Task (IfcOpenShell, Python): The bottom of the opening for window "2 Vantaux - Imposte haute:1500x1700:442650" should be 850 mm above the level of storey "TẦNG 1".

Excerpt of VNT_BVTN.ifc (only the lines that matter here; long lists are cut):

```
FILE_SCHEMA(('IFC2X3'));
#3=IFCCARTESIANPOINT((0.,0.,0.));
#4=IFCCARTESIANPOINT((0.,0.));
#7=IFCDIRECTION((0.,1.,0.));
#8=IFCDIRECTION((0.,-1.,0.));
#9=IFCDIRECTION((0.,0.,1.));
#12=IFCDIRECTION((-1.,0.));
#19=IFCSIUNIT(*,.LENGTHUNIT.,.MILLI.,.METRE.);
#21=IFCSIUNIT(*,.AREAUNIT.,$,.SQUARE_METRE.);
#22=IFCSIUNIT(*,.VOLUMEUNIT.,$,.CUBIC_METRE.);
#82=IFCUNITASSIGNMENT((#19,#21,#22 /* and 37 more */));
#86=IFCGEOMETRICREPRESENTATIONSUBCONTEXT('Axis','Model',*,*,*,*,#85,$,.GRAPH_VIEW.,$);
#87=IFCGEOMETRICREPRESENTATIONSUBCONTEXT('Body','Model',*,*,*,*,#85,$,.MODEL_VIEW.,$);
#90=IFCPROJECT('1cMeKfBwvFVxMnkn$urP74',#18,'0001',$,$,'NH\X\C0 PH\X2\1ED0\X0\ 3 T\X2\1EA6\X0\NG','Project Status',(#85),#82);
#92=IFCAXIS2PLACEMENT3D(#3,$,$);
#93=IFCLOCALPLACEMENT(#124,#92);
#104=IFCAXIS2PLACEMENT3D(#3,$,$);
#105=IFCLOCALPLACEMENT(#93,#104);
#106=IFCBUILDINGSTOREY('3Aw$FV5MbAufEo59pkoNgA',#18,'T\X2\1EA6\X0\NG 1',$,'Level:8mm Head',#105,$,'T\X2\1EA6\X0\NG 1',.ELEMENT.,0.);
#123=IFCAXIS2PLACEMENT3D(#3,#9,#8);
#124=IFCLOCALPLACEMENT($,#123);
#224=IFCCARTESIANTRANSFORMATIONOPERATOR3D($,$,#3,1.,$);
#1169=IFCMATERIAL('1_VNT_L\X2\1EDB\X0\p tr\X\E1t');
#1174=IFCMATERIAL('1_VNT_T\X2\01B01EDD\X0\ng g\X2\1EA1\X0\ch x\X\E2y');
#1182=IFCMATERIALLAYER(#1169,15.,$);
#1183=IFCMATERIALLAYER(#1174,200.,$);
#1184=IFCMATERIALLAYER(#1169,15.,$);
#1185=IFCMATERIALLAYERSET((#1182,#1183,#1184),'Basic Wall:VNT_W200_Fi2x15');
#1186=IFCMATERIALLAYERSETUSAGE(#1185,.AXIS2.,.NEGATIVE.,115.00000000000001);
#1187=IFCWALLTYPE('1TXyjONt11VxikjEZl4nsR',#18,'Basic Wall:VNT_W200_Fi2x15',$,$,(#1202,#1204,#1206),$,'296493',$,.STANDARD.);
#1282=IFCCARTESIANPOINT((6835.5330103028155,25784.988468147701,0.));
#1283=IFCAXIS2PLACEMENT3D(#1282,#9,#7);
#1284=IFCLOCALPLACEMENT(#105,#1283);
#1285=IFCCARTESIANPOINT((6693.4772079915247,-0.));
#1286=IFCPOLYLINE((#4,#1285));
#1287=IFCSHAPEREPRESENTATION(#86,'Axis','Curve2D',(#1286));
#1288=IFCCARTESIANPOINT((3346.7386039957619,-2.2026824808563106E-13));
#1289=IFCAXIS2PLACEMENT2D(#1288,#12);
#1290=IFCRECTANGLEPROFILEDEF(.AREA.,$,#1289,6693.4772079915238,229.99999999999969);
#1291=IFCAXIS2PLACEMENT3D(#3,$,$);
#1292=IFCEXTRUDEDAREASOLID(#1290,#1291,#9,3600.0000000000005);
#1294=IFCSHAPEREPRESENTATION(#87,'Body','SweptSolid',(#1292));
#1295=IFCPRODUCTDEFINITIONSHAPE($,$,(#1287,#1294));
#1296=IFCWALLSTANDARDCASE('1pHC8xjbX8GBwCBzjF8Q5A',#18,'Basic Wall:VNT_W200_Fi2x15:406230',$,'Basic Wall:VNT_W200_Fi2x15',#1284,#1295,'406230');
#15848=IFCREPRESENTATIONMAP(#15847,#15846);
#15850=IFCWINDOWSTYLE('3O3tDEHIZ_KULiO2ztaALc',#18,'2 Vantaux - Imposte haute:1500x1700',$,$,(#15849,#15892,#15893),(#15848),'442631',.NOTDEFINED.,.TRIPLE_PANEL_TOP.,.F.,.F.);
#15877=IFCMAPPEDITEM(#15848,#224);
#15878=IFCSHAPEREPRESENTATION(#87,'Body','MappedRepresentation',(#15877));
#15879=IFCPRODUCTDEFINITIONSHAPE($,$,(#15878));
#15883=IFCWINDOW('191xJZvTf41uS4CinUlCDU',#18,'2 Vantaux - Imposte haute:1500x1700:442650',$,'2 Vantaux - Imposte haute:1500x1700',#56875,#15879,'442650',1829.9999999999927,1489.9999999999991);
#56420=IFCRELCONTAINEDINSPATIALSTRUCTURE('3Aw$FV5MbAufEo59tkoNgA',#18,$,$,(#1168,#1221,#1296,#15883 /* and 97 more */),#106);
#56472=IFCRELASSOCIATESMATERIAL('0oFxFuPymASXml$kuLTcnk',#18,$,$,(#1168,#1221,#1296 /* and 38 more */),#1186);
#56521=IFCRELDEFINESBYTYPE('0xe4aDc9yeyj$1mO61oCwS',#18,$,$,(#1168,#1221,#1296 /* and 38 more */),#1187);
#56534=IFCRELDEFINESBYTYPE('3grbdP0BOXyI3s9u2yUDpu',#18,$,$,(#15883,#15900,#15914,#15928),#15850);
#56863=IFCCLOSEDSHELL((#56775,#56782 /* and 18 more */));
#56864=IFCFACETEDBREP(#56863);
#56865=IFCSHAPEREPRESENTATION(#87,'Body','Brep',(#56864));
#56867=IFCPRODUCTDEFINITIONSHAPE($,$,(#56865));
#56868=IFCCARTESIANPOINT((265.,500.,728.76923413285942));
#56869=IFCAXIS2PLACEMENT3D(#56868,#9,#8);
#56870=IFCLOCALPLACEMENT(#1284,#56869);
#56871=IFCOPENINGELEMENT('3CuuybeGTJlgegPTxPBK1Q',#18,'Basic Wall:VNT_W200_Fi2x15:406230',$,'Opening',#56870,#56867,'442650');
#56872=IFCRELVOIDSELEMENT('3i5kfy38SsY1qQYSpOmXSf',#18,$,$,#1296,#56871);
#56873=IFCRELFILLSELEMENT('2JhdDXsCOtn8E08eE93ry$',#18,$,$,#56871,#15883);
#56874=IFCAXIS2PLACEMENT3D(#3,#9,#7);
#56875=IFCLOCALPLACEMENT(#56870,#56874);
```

```python
import numpy as np
import ifcopenshell
import ifcopenshell.api.geometry
import ifcopenshell.geom
import ifcopenshell.util.element
import ifcopenshell.util.placement
import ifcopenshell.util.shape
import ifcopenshell.util.unit

model = ifcopenshell.open("VNT_BVTN.ifc")
unit_scale = ifcopenshell.util.unit.calculate_unit_scale(model)

window = model.by_guid("191xJZvTf41uS4CinUlCDU")
opening = window.FillsVoids[0].RelatingOpeningElement
storey = ifcopenshell.util.element.get_container(window, ifc_class="IfcBuildingStorey")
level = ifcopenshell.util.placement.get_local_placement(storey.ObjectPlacement)[2, 3]

# The opening's origin need not be at the sill, so measure its lowest point.
shape = ifcopenshell.geom.create_shape(ifcopenshell.geom.settings(), opening)
bottom = ifcopenshell.util.shape.get_shape_bottom_elevation(shape, shape.geometry) / unit_scale
dz = level + 850.0 - bottom

shift = np.array([0.0, 0.0, dz])
# The window is placed relative to its opening, so it follows when the opening moves.
matrix = ifcopenshell.util.placement.get_local_placement(opening.ObjectPlacement)
matrix[:3, 3] += shift
ifcopenshell.api.geometry.edit_object_placement(
    model, product=opening, matrix=matrix, is_si=False, should_transform_children=True
)

print(f"moved by {dz * unit_scale:+.3f} m")

model.write("VNT_BVTN_v2.ifc")
```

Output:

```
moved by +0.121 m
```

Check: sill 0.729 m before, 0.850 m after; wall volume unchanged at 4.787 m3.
